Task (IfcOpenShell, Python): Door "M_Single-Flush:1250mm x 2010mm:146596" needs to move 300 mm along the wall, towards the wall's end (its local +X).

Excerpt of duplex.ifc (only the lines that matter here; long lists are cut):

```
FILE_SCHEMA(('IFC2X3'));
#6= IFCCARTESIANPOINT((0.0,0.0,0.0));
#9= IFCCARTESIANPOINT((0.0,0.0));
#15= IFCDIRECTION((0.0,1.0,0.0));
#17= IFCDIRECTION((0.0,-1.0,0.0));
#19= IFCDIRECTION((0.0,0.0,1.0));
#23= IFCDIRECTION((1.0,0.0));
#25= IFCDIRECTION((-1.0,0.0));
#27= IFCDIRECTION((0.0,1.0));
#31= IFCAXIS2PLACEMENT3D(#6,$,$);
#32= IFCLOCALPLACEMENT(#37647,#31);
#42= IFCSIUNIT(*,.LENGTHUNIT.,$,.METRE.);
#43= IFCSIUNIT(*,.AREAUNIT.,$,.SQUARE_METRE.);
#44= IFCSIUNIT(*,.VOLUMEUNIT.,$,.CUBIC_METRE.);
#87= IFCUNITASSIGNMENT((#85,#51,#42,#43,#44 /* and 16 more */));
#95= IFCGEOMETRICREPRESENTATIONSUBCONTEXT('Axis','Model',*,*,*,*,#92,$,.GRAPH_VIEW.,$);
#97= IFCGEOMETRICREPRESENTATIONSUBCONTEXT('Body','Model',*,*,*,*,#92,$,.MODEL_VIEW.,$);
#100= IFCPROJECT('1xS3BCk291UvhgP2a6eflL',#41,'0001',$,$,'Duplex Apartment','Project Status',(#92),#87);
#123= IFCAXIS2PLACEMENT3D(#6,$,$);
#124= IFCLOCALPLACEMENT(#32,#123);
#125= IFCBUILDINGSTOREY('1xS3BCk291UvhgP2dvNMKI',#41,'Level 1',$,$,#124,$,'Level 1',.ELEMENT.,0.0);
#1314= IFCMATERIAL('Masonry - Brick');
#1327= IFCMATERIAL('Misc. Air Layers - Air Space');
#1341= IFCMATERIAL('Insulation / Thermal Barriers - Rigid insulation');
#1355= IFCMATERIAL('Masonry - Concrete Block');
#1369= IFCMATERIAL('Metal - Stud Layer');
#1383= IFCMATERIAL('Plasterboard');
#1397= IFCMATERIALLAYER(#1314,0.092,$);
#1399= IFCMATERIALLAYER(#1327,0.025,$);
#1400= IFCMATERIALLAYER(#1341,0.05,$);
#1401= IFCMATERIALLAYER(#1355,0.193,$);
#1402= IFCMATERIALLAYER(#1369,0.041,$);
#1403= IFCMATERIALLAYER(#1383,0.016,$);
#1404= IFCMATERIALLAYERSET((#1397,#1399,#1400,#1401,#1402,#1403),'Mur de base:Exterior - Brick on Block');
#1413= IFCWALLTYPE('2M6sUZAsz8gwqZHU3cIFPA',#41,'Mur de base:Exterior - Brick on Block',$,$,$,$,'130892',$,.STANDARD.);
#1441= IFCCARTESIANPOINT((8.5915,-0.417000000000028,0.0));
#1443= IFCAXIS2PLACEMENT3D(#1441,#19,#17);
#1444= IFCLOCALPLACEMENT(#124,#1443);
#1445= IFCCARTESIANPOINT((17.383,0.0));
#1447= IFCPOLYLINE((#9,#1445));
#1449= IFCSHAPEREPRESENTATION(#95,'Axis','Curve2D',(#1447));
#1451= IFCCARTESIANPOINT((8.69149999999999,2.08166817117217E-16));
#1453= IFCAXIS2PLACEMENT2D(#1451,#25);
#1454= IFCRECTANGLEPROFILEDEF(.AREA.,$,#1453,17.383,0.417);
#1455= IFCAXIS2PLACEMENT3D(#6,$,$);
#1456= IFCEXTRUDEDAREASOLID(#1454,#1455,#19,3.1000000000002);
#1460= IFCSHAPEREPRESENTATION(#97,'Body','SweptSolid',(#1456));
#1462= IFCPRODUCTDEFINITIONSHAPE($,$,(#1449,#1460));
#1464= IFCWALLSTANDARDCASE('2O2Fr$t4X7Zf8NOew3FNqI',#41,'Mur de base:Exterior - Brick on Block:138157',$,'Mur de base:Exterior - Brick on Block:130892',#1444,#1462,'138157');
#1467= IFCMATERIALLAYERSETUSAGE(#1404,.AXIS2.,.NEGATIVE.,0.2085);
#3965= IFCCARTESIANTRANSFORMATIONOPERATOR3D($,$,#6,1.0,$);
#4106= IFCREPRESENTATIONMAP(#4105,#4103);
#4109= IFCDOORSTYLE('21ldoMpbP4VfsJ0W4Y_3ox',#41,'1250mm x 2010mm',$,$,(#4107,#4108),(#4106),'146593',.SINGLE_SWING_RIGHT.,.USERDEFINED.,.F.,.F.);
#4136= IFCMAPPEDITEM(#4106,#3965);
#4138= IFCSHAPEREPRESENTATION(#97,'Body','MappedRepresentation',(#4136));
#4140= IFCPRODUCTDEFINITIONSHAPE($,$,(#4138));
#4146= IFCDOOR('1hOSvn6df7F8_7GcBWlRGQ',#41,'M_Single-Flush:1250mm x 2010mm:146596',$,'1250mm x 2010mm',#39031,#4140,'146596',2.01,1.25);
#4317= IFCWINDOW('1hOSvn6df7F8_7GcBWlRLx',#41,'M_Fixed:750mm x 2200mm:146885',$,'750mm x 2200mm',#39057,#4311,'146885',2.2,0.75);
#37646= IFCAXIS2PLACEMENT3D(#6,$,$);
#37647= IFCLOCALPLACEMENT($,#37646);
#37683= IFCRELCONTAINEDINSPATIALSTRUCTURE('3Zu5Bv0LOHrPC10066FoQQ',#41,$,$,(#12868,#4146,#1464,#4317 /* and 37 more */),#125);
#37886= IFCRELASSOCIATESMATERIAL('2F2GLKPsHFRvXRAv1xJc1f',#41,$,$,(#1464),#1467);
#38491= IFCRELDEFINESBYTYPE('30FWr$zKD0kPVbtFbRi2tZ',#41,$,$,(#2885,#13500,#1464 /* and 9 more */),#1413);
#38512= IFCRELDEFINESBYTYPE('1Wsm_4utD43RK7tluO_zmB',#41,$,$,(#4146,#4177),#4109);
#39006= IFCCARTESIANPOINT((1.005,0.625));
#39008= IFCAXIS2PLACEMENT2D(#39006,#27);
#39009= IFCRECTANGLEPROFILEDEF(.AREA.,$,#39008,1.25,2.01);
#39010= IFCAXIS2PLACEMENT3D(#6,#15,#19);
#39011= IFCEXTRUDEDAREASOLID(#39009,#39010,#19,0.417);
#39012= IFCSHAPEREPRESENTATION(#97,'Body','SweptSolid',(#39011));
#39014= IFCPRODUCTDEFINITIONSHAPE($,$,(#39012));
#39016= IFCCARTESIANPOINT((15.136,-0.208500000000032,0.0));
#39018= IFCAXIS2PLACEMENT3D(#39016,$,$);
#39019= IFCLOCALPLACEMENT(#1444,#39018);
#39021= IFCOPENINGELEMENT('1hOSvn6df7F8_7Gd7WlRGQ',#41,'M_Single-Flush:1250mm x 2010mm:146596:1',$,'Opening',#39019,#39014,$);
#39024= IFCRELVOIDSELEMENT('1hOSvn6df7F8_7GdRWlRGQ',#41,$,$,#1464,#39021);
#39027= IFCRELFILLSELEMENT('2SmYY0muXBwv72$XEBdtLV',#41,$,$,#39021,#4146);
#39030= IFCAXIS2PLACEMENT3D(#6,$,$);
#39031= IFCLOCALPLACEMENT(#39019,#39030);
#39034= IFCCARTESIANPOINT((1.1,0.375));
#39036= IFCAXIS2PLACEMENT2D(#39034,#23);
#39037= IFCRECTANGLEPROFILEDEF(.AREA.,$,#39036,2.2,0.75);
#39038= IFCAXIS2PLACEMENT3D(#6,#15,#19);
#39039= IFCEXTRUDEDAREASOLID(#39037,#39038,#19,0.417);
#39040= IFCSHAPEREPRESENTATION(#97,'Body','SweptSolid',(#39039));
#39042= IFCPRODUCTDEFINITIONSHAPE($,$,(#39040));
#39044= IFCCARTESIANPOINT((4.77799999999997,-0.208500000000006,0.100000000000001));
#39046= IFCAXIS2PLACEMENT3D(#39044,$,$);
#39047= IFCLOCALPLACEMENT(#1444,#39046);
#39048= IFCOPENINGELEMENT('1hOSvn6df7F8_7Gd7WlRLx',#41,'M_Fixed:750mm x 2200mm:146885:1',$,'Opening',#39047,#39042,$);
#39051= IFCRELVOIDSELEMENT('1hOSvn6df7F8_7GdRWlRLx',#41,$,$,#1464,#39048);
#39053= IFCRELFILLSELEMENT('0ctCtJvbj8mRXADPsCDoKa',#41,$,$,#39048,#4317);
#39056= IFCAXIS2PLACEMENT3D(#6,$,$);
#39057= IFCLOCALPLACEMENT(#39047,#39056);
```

```python
import ifcopenshell
import ifcopenshell.api.geometry
import ifcopenshell.util.placement

model = ifcopenshell.open("duplex.ifc")

door = model.by_guid("1hOSvn6df7F8_7GcBWlRGQ")
opening = door.FillsVoids[0].RelatingOpeningElement
wall = opening.VoidsElements[0].RelatingBuildingElement

wall_matrix = ifcopenshell.util.placement.get_local_placement(wall.ObjectPlacement)
shift = wall_matrix[:3, 0] * 0.3
before = ifcopenshell.util.placement.get_local_placement(door.ObjectPlacement)[:3, 3].copy()

# The door is placed relative to its opening, so it follows when the opening moves.
matrix = ifcopenshell.util.placement.get_local_placement(opening.ObjectPlacement)
matrix[:3, 3] += shift
ifcopenshell.api.geometry.edit_object_placement(
    model, product=opening, matrix=matrix, is_si=False, should_transform_children=True
)

after = ifcopenshell.util.placement.get_local_placement(door.ObjectPlacement)[:3, 3]
print("door moved by", (after - before).round(3) + 0.0)

model.write("duplex_v2.ifc")
```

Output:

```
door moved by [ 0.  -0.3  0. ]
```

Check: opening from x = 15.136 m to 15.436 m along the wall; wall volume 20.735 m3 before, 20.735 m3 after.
